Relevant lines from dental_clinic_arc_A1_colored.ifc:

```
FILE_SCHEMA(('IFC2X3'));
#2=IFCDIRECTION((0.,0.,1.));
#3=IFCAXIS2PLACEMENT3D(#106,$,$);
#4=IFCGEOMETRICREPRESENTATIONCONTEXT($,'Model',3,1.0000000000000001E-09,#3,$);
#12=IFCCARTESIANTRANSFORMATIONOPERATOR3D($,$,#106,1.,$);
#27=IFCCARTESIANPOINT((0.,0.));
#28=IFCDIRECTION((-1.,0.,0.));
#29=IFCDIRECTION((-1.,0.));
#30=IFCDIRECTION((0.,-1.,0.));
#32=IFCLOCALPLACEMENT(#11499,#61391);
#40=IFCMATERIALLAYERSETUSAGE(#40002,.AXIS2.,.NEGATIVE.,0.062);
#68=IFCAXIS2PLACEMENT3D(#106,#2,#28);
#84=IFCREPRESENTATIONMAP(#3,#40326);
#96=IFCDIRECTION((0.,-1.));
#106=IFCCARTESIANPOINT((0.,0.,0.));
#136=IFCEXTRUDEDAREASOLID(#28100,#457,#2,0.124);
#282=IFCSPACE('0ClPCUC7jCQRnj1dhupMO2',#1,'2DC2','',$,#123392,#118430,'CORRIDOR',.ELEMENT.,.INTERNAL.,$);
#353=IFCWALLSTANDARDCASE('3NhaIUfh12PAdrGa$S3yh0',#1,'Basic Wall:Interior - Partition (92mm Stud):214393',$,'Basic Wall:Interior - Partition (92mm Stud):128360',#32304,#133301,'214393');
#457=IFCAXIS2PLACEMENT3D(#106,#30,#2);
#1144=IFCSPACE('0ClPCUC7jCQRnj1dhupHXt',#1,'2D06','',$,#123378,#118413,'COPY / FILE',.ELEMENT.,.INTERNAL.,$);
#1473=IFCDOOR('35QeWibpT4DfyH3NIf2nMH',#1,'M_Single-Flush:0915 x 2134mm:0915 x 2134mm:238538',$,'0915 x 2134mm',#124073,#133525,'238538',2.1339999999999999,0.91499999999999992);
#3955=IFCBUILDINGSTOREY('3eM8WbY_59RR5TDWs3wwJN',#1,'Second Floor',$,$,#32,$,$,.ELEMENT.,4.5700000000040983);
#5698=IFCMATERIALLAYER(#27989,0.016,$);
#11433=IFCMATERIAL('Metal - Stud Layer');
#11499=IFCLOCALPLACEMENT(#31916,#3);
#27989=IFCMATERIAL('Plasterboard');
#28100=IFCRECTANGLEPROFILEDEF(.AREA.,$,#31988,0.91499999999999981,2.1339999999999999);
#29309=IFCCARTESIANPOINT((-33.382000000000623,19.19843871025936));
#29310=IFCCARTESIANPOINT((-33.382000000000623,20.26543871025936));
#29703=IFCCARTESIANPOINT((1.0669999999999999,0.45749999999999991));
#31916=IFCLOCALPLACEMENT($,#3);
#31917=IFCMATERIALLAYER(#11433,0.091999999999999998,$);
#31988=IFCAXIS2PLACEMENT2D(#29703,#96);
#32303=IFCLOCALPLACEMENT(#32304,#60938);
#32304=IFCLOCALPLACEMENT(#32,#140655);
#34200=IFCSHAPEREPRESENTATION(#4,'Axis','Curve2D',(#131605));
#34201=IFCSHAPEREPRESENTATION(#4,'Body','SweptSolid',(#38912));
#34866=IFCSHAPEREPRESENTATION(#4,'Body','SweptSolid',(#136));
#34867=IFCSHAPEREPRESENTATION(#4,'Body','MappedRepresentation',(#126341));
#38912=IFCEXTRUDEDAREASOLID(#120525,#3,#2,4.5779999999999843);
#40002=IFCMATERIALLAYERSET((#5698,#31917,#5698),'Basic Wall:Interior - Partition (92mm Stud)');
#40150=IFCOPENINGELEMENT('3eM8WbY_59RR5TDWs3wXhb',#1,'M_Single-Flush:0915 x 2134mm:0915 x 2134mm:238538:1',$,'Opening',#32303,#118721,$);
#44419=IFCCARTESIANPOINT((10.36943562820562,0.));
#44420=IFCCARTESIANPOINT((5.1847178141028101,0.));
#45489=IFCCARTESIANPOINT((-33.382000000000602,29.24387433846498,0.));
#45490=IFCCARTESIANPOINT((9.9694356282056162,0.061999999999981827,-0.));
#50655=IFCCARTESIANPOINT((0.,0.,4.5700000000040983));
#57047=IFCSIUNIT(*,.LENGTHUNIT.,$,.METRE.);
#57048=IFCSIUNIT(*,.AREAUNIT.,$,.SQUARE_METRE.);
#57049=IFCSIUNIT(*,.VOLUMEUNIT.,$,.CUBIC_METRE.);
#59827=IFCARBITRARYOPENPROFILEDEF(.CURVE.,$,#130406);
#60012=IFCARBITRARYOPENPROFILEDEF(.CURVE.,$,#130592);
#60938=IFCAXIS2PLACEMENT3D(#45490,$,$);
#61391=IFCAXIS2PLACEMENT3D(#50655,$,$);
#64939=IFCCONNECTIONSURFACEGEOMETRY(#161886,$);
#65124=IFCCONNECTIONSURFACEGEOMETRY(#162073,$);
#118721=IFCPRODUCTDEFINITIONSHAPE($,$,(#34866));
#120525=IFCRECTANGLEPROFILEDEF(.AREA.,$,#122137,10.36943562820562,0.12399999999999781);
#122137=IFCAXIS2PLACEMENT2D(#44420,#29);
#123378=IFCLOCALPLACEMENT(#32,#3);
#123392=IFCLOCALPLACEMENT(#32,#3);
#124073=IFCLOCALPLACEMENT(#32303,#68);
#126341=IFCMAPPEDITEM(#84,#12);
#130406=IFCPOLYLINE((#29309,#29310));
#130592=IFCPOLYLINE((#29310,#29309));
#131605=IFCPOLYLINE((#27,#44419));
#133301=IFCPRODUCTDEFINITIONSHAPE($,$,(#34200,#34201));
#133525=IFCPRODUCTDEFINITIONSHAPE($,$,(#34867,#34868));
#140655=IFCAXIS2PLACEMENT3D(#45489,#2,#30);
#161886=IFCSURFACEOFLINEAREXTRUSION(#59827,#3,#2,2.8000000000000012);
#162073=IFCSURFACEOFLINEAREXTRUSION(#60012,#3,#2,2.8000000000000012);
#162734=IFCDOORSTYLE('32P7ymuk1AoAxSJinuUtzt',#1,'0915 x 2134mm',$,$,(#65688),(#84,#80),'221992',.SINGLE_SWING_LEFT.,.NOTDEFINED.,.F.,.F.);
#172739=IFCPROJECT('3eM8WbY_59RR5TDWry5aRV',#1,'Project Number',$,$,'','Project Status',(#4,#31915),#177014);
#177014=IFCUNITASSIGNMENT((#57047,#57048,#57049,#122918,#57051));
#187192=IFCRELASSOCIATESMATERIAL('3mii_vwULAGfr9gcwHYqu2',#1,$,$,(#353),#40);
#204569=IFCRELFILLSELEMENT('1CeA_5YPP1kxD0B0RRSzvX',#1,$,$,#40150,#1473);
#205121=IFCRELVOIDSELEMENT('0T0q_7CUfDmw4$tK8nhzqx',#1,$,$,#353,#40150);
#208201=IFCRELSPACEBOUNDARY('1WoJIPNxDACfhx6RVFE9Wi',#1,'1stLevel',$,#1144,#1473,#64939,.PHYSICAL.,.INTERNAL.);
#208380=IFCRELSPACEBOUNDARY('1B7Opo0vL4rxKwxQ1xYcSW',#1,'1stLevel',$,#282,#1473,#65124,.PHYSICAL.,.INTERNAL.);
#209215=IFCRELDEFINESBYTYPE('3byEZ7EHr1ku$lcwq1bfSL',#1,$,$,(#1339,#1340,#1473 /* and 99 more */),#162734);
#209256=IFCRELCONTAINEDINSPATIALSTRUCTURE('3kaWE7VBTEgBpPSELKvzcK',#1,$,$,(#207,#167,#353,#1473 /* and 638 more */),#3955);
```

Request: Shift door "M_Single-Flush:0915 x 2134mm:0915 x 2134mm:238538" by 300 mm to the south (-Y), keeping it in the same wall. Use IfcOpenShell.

```python
import numpy as np
import ifcopenshell
import ifcopenshell.api.geometry
import ifcopenshell.util.placement

model = ifcopenshell.open("dental_clinic_arc_A1_colored.ifc")

door = model.by_id(1473)
opening = door.FillsVoids[0].RelatingOpeningElement
wall = opening.VoidsElements[0].RelatingBuildingElement

wall_matrix = ifcopenshell.util.placement.get_local_placement(wall.ObjectPlacement)
shift = wall_matrix[:3, 0] * 0.3
before = ifcopenshell.util.placement.get_local_placement(door.ObjectPlacement)[:3, 3].copy()

# The door is placed relative to its opening, so it follows when the opening moves.
matrix = ifcopenshell.util.placement.get_local_placement(opening.ObjectPlacement)
matrix[:3, 3] += shift
ifcopenshell.api.geometry.edit_object_placement(
    model, product=opening, matrix=matrix, is_si=False, should_transform_children=True
)

# Space boundary surfaces are stored in each space's coordinates; move them too.
for rel in door.ProvidesBoundaries:
    if not rel.ConnectionGeometry:
        continue
    surface = rel.ConnectionGeometry.SurfaceOnRelatingElement
    space_matrix = ifcopenshell.util.placement.get_local_placement(rel.RelatingSpace.ObjectPlacement)
    point = np.array(surface.Position.Location.Coordinates) + space_matrix[:3, :3].T @ shift
    surface.Position = model.createIfcAxis2Placement3D(
        model.createIfcCartesianPoint(point.tolist()), surface.Position.Axis, surface.Position.RefDirection
    )

after = ifcopenshell.util.placement.get_local_placement(door.ObjectPlacement)[:3, 3]
print("door moved by", (after - before).round(3) + 0.0)

model.write("dental_clinic_arc_A1_colored_edited.ifc")
```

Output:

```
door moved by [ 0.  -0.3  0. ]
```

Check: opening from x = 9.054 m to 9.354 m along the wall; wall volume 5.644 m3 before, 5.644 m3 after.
